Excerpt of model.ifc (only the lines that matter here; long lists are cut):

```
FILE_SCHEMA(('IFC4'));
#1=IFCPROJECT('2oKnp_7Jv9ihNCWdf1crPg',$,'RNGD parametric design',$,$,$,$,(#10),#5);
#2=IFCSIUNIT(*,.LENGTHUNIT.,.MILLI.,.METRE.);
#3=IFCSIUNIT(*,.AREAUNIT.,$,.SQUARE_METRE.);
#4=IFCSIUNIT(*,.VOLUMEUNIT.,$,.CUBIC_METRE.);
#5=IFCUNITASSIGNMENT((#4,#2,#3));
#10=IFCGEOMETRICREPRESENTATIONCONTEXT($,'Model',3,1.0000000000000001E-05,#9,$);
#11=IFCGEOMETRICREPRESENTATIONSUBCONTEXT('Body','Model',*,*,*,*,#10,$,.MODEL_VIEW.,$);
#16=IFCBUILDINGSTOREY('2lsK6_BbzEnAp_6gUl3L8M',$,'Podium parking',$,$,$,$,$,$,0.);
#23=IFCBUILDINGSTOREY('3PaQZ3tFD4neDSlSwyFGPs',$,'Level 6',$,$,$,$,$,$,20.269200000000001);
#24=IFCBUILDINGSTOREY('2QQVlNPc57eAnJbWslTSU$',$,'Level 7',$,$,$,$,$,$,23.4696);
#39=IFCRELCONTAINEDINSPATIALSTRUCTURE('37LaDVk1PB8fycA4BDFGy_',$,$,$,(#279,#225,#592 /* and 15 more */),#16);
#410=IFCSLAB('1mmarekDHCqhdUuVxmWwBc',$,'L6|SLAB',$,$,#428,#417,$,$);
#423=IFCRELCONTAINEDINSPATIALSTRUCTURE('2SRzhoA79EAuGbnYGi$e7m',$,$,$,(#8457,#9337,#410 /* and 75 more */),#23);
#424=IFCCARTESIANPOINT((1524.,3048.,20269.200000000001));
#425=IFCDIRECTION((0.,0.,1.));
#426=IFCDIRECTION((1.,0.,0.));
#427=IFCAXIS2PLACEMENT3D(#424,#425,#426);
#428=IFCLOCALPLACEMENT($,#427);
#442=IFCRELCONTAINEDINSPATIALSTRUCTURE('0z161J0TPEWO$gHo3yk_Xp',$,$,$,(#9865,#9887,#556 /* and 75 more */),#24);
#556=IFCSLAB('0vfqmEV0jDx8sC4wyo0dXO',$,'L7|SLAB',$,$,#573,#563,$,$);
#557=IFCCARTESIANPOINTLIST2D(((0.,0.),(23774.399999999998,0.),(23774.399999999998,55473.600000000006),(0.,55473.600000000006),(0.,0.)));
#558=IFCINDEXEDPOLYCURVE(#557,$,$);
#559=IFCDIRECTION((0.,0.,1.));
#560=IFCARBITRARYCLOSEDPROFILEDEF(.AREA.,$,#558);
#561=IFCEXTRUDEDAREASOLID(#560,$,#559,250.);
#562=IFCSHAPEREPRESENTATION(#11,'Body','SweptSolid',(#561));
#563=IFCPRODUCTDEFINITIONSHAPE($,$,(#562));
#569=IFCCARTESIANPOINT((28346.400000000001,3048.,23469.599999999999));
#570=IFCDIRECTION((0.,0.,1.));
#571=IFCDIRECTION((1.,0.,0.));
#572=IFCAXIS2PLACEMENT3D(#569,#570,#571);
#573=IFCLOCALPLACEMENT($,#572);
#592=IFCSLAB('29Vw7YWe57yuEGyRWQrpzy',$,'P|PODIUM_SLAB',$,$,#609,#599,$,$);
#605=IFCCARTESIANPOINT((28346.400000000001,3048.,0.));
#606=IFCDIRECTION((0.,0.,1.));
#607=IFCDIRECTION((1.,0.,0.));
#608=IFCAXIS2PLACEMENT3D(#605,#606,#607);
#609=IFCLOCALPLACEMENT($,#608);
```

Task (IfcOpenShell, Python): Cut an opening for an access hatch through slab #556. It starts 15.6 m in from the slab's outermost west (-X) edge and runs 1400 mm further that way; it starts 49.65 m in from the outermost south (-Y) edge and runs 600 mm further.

```python
import numpy as np
import ifcopenshell
import ifcopenshell.api.feature
import ifcopenshell.api.geometry
import ifcopenshell.api.root
import ifcopenshell.geom
import ifcopenshell.util.placement
import ifcopenshell.util.representation
import ifcopenshell.util.shape
import ifcopenshell.util.unit

model = ifcopenshell.open("model.ifc")
unit_scale = ifcopenshell.util.unit.calculate_unit_scale(model)
settings = ifcopenshell.geom.settings()


def volume(element):
    """Net volume in cubic metres, openings subtracted."""
    shape = ifcopenshell.geom.create_shape(settings, element)
    return ifcopenshell.util.shape.get_volume(shape.geometry)


slab = model.by_id(556)
before = volume(slab)

# Extent in the slab's own axes, in metres. The edges named are its -X and -Y sides.
slab_shape = ifcopenshell.geom.create_shape(settings, slab)
vertices = ifcopenshell.util.shape.get_vertices(slab_shape.geometry)
x_min, y_min, bottom = vertices.min(axis=0)
top = vertices[:, 2].max()

opening = ifcopenshell.api.root.create_entity(model, ifc_class="IfcOpeningElement", name="Access hatch opening", predefined_type="OPENING")
context = ifcopenshell.util.representation.get_context(model, "Model", "Body", "MODEL_VIEW")
width, depth = 1.4, 0.6
outline = [(0.0, 0.0), (width, 0.0), (width, depth), (0.0, depth), (0.0, 0.0)]
# Overshoot both faces by 50 mm so the cut is clean.
shape = ifcopenshell.api.geometry.add_slab_representation(
    model, context=context, depth=top - bottom + 0.1, polyline=outline
)
ifcopenshell.api.geometry.assign_representation(model, product=opening, representation=shape)

matrix = ifcopenshell.util.placement.get_local_placement(slab.ObjectPlacement)
matrix[:, 3] = matrix @ np.append(np.array([x_min + 15.6, y_min + 49.65, bottom - 0.05]) / unit_scale, 1.0)
ifcopenshell.api.geometry.edit_object_placement(model, product=opening, matrix=matrix, is_si=False)
ifcopenshell.api.feature.add_feature(model, feature=opening, element=slab)

after = volume(slab)

print(f"slab volume {before:.3f} -> {after:.3f} m3")

model.write("model_rev.ifc")
```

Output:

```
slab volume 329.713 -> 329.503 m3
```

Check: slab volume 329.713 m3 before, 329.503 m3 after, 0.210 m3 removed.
